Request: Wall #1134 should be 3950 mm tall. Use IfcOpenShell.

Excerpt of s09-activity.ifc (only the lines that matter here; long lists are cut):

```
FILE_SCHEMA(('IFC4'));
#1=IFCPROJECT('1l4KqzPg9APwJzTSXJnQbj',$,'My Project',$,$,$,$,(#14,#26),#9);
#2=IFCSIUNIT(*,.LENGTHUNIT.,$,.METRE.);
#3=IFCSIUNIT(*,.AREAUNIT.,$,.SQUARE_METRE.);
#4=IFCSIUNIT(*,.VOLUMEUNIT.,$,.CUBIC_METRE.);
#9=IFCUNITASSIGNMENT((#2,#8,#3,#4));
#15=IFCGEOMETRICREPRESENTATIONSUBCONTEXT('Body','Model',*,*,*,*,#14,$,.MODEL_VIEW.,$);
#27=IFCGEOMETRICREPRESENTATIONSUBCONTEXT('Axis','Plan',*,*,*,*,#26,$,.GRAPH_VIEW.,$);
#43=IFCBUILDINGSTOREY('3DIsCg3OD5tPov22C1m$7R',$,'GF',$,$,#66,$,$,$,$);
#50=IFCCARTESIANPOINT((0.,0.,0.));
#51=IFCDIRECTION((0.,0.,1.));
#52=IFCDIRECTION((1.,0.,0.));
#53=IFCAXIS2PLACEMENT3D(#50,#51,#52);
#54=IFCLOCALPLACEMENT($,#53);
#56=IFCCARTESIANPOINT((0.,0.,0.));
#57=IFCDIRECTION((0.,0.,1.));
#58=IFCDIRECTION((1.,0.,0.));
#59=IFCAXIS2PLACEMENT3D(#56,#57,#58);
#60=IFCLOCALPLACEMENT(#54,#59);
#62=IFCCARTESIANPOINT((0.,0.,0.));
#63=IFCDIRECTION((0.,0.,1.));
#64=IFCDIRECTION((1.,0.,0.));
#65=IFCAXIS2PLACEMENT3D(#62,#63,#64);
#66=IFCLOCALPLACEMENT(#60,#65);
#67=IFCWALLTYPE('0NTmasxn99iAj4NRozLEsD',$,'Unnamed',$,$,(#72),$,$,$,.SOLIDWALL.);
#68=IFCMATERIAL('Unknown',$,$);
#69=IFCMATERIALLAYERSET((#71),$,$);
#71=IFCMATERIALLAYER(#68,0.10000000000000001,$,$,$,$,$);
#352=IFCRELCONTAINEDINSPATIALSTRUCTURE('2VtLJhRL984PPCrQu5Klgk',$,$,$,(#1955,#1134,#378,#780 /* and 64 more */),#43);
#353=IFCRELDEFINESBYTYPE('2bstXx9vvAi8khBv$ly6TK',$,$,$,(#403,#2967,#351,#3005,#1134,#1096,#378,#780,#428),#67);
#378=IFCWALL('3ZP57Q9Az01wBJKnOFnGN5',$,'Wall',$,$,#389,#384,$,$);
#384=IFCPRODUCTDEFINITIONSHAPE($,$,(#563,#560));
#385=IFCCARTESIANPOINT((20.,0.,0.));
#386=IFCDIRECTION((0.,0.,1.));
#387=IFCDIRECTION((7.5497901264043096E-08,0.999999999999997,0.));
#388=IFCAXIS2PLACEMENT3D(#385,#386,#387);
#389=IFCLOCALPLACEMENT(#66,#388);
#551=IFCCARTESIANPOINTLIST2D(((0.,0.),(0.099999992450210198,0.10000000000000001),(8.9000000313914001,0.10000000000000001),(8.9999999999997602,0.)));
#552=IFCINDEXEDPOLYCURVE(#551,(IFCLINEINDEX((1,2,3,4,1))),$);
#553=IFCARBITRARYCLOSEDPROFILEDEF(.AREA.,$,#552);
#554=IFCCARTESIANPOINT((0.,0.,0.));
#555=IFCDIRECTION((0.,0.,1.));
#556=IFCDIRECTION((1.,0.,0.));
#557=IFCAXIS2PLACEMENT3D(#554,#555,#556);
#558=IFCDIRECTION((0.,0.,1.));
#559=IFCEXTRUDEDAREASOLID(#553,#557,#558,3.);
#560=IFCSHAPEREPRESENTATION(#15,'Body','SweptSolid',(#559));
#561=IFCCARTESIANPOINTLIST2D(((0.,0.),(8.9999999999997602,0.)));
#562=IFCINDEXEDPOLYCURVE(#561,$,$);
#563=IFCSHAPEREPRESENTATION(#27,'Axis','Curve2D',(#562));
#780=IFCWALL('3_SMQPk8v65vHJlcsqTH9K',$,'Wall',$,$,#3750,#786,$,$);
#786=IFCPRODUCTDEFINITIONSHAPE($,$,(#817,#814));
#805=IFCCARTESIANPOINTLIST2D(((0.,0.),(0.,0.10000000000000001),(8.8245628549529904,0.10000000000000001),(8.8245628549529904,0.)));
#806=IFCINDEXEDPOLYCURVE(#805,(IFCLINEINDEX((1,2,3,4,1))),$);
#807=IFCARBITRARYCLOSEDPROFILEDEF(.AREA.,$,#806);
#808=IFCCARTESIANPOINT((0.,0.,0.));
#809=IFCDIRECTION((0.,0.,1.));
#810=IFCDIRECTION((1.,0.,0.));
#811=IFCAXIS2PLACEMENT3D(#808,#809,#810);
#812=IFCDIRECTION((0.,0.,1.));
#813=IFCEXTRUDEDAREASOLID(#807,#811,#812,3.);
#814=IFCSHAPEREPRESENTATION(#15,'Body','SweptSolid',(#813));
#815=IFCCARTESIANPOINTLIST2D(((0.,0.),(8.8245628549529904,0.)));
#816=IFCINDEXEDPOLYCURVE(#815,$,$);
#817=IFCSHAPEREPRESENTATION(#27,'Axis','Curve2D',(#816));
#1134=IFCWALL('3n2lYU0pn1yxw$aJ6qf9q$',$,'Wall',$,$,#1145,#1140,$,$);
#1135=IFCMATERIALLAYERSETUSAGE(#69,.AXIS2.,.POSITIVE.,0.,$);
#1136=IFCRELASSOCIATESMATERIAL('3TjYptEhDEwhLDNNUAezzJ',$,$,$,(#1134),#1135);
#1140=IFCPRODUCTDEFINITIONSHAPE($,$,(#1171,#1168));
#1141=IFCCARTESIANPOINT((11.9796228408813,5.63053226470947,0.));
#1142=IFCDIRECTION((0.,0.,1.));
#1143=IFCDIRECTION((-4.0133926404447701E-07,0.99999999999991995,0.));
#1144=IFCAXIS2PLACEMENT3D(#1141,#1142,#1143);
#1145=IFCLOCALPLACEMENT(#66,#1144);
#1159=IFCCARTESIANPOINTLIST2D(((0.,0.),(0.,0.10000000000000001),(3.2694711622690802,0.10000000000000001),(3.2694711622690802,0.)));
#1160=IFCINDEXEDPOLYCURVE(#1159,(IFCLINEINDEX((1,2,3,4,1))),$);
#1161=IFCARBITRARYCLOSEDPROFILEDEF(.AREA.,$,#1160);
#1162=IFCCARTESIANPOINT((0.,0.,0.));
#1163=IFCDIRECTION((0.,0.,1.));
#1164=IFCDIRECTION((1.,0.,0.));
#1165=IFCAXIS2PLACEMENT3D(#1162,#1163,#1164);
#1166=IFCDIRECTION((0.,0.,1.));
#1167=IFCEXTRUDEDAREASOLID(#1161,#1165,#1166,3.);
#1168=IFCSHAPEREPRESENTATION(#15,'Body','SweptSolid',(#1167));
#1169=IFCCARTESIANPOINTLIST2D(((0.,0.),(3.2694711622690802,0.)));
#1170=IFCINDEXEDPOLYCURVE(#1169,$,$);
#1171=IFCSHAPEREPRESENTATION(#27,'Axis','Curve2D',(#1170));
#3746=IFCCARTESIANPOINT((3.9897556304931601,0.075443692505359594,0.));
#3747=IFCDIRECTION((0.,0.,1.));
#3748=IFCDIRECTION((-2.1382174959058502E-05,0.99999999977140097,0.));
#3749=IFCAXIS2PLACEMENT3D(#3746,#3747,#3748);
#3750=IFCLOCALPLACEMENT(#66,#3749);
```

```python
import ifcopenshell
import ifcopenshell.geom
import ifcopenshell.util.representation
import ifcopenshell.util.shape

model = ifcopenshell.open("s09-activity.ifc")
settings = ifcopenshell.geom.settings()


def volume(element):
    """Net volume in cubic metres, openings subtracted."""
    shape = ifcopenshell.geom.create_shape(settings, element)
    return ifcopenshell.util.shape.get_volume(shape.geometry)


wall = model.by_guid("3n2lYU0pn1yxw$aJ6qf9q$")
before = volume(wall)

body = ifcopenshell.util.representation.get_representation(wall, "Model", "Body")
solid = body.Items[0]
old_height = solid.Depth
solid.Depth = 3.95
after = volume(wall)

print(f"height {old_height:g} -> {solid.Depth:g}, volume {before:.3f} -> {after:.3f} m3")

model.write("s09-activity_edited.ifc")
```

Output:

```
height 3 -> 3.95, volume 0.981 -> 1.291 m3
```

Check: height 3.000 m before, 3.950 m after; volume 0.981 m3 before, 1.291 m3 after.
